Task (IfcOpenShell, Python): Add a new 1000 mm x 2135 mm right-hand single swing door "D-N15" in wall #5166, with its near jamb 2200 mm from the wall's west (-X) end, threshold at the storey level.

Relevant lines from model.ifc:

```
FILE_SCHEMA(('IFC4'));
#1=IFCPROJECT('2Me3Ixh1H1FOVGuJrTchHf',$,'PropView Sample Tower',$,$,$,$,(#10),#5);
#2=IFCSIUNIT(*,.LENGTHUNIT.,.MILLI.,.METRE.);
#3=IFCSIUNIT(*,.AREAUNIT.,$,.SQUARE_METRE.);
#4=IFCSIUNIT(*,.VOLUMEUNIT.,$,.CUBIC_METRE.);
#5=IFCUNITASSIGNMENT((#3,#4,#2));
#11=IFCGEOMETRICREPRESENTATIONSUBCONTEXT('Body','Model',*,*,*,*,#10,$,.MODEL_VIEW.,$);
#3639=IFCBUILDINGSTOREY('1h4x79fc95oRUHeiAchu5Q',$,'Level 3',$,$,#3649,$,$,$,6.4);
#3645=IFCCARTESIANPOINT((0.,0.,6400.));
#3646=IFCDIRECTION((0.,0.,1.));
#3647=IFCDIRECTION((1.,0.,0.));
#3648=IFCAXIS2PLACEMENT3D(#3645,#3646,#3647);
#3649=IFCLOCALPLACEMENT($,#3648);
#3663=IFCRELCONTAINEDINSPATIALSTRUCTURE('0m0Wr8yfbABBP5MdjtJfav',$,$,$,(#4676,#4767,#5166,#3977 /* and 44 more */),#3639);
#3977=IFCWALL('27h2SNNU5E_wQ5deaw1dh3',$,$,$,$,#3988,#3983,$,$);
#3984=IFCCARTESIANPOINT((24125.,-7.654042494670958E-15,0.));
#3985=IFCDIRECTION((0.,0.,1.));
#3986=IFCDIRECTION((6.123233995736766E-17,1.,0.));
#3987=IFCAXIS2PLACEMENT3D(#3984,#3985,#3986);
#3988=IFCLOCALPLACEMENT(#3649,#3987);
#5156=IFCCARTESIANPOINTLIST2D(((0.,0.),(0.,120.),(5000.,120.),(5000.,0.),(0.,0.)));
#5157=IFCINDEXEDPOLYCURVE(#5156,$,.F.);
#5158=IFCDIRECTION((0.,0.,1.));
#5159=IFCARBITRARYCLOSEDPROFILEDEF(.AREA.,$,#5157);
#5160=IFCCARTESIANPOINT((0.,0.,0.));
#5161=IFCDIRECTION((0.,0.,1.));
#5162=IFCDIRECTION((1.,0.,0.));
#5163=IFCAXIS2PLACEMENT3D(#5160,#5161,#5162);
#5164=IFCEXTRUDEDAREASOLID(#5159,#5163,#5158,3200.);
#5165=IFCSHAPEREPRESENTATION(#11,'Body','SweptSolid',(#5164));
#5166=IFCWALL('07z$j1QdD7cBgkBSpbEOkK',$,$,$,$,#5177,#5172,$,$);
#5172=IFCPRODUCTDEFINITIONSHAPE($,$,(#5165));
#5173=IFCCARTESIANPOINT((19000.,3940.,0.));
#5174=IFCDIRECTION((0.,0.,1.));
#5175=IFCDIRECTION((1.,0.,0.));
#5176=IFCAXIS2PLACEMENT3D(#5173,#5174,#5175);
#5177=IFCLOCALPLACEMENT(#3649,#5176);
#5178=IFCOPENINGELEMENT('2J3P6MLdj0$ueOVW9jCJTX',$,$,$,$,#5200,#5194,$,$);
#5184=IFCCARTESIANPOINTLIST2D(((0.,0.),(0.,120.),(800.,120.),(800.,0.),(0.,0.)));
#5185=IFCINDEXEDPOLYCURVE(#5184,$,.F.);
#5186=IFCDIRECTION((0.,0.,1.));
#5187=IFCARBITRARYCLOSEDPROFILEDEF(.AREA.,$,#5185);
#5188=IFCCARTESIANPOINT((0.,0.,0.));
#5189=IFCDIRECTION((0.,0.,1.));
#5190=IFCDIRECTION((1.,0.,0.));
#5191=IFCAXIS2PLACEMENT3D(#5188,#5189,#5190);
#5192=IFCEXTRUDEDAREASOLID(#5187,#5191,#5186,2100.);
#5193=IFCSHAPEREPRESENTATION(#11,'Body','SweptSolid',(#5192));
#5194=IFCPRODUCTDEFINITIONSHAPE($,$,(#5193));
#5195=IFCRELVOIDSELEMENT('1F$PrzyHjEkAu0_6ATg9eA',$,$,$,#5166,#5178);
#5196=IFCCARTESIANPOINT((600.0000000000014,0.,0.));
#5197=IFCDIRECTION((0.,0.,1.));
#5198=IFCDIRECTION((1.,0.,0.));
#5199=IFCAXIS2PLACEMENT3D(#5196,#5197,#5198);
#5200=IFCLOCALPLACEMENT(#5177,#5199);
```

```python
import numpy as np
import ifcopenshell
import ifcopenshell.api.feature
import ifcopenshell.api.geometry
import ifcopenshell.api.root
import ifcopenshell.api.spatial
import ifcopenshell.geom
import ifcopenshell.util.element
import ifcopenshell.util.placement
import ifcopenshell.util.representation
import ifcopenshell.util.shape
import ifcopenshell.util.unit

model = ifcopenshell.open("model.ifc")
unit_scale = ifcopenshell.util.unit.calculate_unit_scale(model)
settings = ifcopenshell.geom.settings()


def volume(element):
    """Net volume in cubic metres, openings subtracted."""
    shape = ifcopenshell.geom.create_shape(settings, element)
    return ifcopenshell.util.shape.get_volume(shape.geometry)


wall = model.by_guid("07z$j1QdD7cBgkBSpbEOkK")
storey = ifcopenshell.util.element.get_container(wall, ifc_class="IfcBuildingStorey")
context = ifcopenshell.util.representation.get_context(model, "Model", "Body", "MODEL_VIEW")
before = volume(wall)

width, height, from_end, sill = 1, 2.135, 2.2, 0.0  # metres

# The wall runs along its own X axis, and the end named is its -X end.
wall_shape = ifcopenshell.geom.create_shape(settings, wall)
x, y, z = ifcopenshell.util.shape.get_vertices(wall_shape.geometry).T
start = x.min() + from_end
face, thickness = float(y.min()), float(y.max() - y.min())
wall_matrix = ifcopenshell.util.placement.get_local_placement(wall.ObjectPlacement)
level = ifcopenshell.util.placement.get_local_placement(storey.ObjectPlacement)[2, 3]


def in_wall(x, y):
    """Placement at x, y metres in the wall's axes, at sill height."""
    matrix = wall_matrix.copy()
    matrix[:, 3] = wall_matrix @ np.array([x / unit_scale, y / unit_scale, 0.0, 1.0])
    matrix[2, 3] = level + sill / unit_scale
    return matrix


# Opening: a box that overshoots both wall faces by 50 mm.
opening = ifcopenshell.api.root.create_entity(model, ifc_class="IfcOpeningElement", predefined_type="OPENING")
box = ifcopenshell.api.geometry.add_wall_representation(
    model, context=context, length=width, height=height, thickness=thickness + 0.1
)
ifcopenshell.api.geometry.assign_representation(model, product=opening, representation=box)
ifcopenshell.api.geometry.edit_object_placement(model, product=opening, matrix=in_wall(start, face - 0.05), is_si=False)
ifcopenshell.api.feature.add_feature(model, feature=opening, element=wall)

door = ifcopenshell.api.root.create_entity(model, ifc_class="IfcDoor", name="D-N15", predefined_type="DOOR")
door.OverallWidth, door.OverallHeight = width / unit_scale, height / unit_scale
door.OperationType = "SINGLE_SWING_RIGHT"
body = ifcopenshell.api.geometry.add_door_representation(
    model,
    context=context,
    overall_width=door.OverallWidth,
    overall_height=door.OverallHeight,
    operation_type="SINGLE_SWING_RIGHT",
    lining_properties={"LiningDepth": thickness / unit_scale, "ThresholdDepth": thickness / unit_scale},
)
ifcopenshell.api.geometry.assign_representation(model, product=door, representation=body)
ifcopenshell.api.spatial.assign_container(model, products=[door], relating_structure=storey)
ifcopenshell.api.feature.add_filling(model, opening=opening, element=door)

# The lining spans the wall, so the door starts at the wall face.
ifcopenshell.api.geometry.edit_object_placement(model, product=door, matrix=in_wall(start, face), is_si=False)

after = volume(wall)

print(f"wall volume {before:.3f} -> {after:.3f} m3")

model.write("model_rev.ifc")
```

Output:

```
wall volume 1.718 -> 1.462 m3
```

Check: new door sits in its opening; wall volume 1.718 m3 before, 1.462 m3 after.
